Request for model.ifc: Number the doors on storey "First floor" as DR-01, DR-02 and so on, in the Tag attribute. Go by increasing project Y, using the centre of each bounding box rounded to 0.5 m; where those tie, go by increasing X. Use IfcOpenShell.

First a look at what the model holds.

```python
import ifcopenshell
import ifcopenshell.util.element
import ifcopenshell.util.placement

model = ifcopenshell.open("model.ifc")
print(model.schema)
storey = next(s for s in model.by_type("IfcBuildingStorey") if s.Name == "First floor")
doors = [e for e in ifcopenshell.util.element.get_decomposition(storey) if e.is_a("IfcDoor")]
for e in sorted(doors, key=lambda e: e.id()):
    origin = ifcopenshell.util.placement.get_local_placement(e.ObjectPlacement)[:3, 3]
    print(e.id(), e.Tag, e.Name, origin.round(2) + 0.0, sep=" | ")
```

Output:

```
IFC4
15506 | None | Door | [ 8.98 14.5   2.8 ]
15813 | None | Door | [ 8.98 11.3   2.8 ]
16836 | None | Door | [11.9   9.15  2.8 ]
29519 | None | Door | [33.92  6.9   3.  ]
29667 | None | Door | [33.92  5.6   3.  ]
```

```python
import ifcopenshell
import ifcopenshell.geom
import ifcopenshell.util.element
import ifcopenshell.util.shape

model = ifcopenshell.open("model.ifc")
settings = ifcopenshell.geom.settings()
settings.set("use-world-coords", True)


def centre(element):
    shape = ifcopenshell.geom.create_shape(settings, element)
    return ifcopenshell.util.shape.get_bbox_centroid(shape.geometry)


storey = next(s for s in model.by_type("IfcBuildingStorey") if s.Name == "First floor")
doors = [e for e in ifcopenshell.util.element.get_decomposition(storey) if e.is_a("IfcDoor")]

# Insertion points can sit at a corner or the storey origin, so sort by the geometry (in metres).
centres = {e: centre(e) for e in doors}
doors.sort(key=lambda e: (round(centres[e][1] / 0.5), centres[e][0]))

for i, e in enumerate(doors, start=1):
    number = f"DR-{i:02d}"
    e.Tag = number
    print(e.id(), number)

model.write("model_rev.ifc")
```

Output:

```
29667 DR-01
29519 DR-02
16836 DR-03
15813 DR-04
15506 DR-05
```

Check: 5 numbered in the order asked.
